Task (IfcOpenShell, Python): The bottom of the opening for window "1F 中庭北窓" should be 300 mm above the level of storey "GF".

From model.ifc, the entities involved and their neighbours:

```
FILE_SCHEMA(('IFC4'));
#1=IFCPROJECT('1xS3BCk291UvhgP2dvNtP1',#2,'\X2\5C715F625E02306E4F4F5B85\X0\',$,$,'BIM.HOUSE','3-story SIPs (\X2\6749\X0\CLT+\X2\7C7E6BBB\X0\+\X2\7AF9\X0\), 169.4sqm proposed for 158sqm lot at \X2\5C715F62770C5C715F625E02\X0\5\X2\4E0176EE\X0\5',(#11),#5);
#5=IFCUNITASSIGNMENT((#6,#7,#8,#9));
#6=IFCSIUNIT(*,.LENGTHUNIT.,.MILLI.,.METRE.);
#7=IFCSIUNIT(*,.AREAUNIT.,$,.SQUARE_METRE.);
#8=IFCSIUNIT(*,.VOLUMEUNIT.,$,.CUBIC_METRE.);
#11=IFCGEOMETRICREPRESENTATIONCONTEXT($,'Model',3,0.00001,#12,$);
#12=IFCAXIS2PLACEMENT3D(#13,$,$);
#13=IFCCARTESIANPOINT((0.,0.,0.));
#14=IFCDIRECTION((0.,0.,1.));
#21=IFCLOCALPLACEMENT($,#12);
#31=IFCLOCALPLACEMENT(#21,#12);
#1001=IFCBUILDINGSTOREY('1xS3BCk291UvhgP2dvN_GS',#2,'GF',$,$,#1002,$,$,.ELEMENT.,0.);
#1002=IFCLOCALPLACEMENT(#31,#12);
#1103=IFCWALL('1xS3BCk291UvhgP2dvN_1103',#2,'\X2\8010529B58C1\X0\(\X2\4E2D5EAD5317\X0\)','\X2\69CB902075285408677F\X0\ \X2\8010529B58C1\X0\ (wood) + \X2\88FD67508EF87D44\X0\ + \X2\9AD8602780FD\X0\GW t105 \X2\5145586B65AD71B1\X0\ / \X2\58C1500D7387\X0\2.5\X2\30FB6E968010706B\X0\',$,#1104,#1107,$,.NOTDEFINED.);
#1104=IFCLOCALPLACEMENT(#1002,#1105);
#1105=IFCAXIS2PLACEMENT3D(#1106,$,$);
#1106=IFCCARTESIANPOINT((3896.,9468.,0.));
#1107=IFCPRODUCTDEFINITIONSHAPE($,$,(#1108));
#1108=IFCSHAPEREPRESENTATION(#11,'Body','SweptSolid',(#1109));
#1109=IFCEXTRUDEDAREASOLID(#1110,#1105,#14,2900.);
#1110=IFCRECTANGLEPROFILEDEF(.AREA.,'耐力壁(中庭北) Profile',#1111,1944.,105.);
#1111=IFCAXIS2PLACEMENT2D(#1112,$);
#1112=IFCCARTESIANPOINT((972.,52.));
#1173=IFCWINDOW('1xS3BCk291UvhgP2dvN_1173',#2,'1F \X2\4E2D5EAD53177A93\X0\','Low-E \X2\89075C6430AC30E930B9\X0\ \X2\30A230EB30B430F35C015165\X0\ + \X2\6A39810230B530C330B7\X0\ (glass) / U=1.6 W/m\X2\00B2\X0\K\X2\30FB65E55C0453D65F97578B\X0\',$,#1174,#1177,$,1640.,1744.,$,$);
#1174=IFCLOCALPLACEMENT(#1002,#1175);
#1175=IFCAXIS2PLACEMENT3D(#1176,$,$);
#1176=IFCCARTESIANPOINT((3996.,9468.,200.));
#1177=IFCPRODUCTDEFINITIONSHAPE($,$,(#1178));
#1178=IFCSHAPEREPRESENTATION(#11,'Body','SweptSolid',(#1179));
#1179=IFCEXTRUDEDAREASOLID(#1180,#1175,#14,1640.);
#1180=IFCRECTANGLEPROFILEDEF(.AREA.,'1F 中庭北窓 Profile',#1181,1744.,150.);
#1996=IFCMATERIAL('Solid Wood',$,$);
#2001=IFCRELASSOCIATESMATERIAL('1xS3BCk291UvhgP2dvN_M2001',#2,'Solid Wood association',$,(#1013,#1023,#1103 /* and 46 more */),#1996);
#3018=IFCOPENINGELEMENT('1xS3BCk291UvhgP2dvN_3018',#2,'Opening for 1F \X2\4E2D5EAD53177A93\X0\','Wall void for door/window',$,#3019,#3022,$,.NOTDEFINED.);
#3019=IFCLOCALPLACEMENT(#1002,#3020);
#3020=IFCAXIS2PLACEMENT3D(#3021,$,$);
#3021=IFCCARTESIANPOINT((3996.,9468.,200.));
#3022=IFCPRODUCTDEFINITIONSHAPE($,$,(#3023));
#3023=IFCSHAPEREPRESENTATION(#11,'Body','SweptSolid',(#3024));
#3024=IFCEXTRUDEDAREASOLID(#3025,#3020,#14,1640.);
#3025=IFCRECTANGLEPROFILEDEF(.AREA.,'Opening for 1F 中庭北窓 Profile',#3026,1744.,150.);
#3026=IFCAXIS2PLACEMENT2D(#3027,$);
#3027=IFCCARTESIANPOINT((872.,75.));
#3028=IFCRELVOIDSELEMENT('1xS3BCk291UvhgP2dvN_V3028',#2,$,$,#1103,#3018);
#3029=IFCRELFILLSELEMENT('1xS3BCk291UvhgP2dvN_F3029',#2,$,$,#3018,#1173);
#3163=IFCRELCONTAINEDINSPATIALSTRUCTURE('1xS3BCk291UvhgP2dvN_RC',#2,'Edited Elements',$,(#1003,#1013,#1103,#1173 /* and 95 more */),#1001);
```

```python
import numpy as np
import ifcopenshell
import ifcopenshell.api.geometry
import ifcopenshell.geom
import ifcopenshell.util.element
import ifcopenshell.util.placement
import ifcopenshell.util.shape
import ifcopenshell.util.unit

model = ifcopenshell.open("model.ifc")
unit_scale = ifcopenshell.util.unit.calculate_unit_scale(model)

window = model.by_id(1173)
opening = window.FillsVoids[0].RelatingOpeningElement
storey = ifcopenshell.util.element.get_container(window, ifc_class="IfcBuildingStorey")
level = ifcopenshell.util.placement.get_local_placement(storey.ObjectPlacement)[2, 3]

# The opening's origin need not be at the sill, so measure its lowest point.
shape = ifcopenshell.geom.create_shape(ifcopenshell.geom.settings(), opening)
bottom = ifcopenshell.util.shape.get_shape_bottom_elevation(shape, shape.geometry) / unit_scale
dz = level + 0.3 / unit_scale - bottom

shift = np.array([0.0, 0.0, dz])
# The window is not placed relative to its opening, so move both.
for product in (opening, window):
    matrix = ifcopenshell.util.placement.get_local_placement(product.ObjectPlacement)
    matrix[:3, 3] += shift
    ifcopenshell.api.geometry.edit_object_placement(model, product=product, matrix=matrix, is_si=False)

print(f"moved by {dz * unit_scale:+.3f} m")

model.write("model_edited.ifc")
```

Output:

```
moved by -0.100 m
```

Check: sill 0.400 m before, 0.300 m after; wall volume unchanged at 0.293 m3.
